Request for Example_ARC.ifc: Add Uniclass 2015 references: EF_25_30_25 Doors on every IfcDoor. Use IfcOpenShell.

First a look at what the model holds.

```python
import ifcopenshell

model = ifcopenshell.open("Example_ARC.ifc")
print(model.schema)
print("classifications:", [c.Name for c in model.by_type("IfcClassification")])
for ifc_class in ("IfcDoor", "IfcRoof", "IfcStair", "IfcWall", "IfcWindow"):
    print(ifc_class, len(model.by_type(ifc_class)))
```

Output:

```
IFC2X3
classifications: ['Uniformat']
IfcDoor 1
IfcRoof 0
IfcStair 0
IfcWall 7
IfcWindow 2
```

```python
import ifcopenshell
import ifcopenshell.api.classification

model = ifcopenshell.open("Example_ARC.ifc")

# IFC2X3 requires Source and Edition and has no link from the project to the system.
system = model.create_entity("IfcClassification", Source="NBS", Edition="2015", Name="Uniclass 2015")

codes = {
    "IfcDoor": ("EF_25_30_25", "Doors"),
}
for ifc_class, (code, name) in codes.items():
    products = model.by_type(ifc_class)
    ifcopenshell.api.classification.add_reference(
        model, products=products, classification=system, identification=code, name=name
    )
    print(code, len(products))

model.write("Example_ARC_v2.ifc")
```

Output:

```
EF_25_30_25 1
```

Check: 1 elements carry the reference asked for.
